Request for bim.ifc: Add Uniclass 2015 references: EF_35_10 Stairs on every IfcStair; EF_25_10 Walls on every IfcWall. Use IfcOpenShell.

First a look at what the model holds.

```python
import ifcopenshell

model = ifcopenshell.open("bim.ifc")
print(model.schema)
print("classifications:", [c.Name for c in model.by_type("IfcClassification")])
for ifc_class in ("IfcDoor", "IfcRoof", "IfcStair", "IfcWall", "IfcWindow"):
    print(ifc_class, len(model.by_type(ifc_class)))
```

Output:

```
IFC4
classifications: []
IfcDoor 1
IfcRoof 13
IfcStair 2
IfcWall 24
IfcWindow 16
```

```python
import ifcopenshell
import ifcopenshell.api.classification

model = ifcopenshell.open("bim.ifc")

system = ifcopenshell.api.classification.add_classification(model, classification="Uniclass 2015")

codes = {
    "IfcStair": ("EF_35_10", "Stairs"),
    "IfcWall": ("EF_25_10", "Walls"),
}
for ifc_class, (code, name) in codes.items():
    products = model.by_type(ifc_class)
    ifcopenshell.api.classification.add_reference(
        model, products=products, classification=system, identification=code, name=name
    )
    print(code, len(products))

model.write("bim-out.ifc")
```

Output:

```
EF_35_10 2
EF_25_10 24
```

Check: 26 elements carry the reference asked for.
